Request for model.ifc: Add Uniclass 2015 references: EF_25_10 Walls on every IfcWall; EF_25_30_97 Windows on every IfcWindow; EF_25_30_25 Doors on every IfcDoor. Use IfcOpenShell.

First a look at what the model holds.

```python
import ifcopenshell

model = ifcopenshell.open("model.ifc")
print(model.schema)
print("classifications:", [c.Name for c in model.by_type("IfcClassification")])
for ifc_class in ("IfcDoor", "IfcRoof", "IfcStair", "IfcWall", "IfcWindow"):
    print(ifc_class, len(model.by_type(ifc_class)))
```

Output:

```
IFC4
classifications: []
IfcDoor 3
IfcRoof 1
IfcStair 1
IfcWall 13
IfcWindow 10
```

```python
import ifcopenshell
import ifcopenshell.api.classification

model = ifcopenshell.open("model.ifc")

system = ifcopenshell.api.classification.add_classification(model, classification="Uniclass 2015")

codes = {
    "IfcWall": ("EF_25_10", "Walls"),
    "IfcWindow": ("EF_25_30_97", "Windows"),
    "IfcDoor": ("EF_25_30_25", "Doors"),
}
for ifc_class, (code, name) in codes.items():
    products = model.by_type(ifc_class)
    ifcopenshell.api.classification.add_reference(
        model, products=products, classification=system, identification=code, name=name
    )
    print(code, len(products))

model.write("model_edited.ifc")
```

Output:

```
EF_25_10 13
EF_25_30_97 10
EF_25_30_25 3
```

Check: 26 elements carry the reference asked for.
